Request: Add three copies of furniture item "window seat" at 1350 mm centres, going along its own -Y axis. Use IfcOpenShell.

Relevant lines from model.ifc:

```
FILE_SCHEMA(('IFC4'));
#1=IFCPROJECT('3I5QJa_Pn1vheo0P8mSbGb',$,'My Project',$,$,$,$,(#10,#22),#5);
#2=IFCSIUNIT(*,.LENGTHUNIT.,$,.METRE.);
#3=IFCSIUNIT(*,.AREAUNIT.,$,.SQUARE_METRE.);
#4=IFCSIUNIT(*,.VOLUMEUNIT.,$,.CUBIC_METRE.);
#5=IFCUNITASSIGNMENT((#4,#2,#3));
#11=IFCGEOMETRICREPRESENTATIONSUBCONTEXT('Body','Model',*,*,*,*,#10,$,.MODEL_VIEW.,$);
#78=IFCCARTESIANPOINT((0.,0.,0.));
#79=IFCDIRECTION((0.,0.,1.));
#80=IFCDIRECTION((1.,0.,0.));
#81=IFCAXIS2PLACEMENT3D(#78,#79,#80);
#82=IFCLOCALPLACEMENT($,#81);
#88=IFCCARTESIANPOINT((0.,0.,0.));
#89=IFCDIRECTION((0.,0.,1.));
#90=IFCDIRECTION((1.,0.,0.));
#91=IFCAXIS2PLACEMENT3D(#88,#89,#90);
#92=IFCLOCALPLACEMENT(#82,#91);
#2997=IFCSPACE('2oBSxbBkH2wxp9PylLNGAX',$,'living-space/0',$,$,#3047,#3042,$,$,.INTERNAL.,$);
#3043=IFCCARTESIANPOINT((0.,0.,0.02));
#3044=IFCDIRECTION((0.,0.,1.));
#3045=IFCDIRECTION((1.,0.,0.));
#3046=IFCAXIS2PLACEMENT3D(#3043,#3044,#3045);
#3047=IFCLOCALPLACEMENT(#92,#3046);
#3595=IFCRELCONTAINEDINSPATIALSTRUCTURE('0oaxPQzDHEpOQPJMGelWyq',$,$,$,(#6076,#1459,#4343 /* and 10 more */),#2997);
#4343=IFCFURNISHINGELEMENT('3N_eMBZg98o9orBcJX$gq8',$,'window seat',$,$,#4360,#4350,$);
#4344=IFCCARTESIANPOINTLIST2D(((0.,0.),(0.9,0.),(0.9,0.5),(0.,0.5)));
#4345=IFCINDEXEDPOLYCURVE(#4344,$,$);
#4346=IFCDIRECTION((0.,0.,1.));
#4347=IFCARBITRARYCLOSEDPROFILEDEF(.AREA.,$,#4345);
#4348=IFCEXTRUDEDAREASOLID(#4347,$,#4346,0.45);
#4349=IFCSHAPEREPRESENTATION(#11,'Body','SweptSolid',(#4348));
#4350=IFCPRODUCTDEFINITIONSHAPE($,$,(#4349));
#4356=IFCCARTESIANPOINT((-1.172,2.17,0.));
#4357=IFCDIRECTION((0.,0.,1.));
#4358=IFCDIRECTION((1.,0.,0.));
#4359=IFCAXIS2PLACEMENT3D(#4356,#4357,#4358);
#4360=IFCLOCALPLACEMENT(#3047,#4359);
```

```python
import ifcopenshell
import ifcopenshell.api.geometry
import ifcopenshell.api.root
import ifcopenshell.util.element
import ifcopenshell.util.placement
import ifcopenshell.util.unit

model = ifcopenshell.open("model.ifc")
unit_scale = ifcopenshell.util.unit.calculate_unit_scale(model)

source = model.by_id(4343)
base = ifcopenshell.util.placement.get_local_placement(source.ObjectPlacement)
step = -base[:3, 1] * 1.35 / unit_scale

for i in range(1, 4):
    copy = ifcopenshell.api.root.copy_class(model, product=source)
    copy.Representation = ifcopenshell.util.element.copy_deep(
        model, source.Representation, exclude=["IfcGeometricRepresentationContext", "IfcRepresentationMap"]
    )
    matrix = base.copy()
    matrix[:3, 3] += i * step
    print("added at", matrix[:3, 3].round(3) + 0.0)
    ifcopenshell.api.geometry.edit_object_placement(model, product=copy, matrix=matrix, is_si=False)

model.write("model_edited.ifc")
```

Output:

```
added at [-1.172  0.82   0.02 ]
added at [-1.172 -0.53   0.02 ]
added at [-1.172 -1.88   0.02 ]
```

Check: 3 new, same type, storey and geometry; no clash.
